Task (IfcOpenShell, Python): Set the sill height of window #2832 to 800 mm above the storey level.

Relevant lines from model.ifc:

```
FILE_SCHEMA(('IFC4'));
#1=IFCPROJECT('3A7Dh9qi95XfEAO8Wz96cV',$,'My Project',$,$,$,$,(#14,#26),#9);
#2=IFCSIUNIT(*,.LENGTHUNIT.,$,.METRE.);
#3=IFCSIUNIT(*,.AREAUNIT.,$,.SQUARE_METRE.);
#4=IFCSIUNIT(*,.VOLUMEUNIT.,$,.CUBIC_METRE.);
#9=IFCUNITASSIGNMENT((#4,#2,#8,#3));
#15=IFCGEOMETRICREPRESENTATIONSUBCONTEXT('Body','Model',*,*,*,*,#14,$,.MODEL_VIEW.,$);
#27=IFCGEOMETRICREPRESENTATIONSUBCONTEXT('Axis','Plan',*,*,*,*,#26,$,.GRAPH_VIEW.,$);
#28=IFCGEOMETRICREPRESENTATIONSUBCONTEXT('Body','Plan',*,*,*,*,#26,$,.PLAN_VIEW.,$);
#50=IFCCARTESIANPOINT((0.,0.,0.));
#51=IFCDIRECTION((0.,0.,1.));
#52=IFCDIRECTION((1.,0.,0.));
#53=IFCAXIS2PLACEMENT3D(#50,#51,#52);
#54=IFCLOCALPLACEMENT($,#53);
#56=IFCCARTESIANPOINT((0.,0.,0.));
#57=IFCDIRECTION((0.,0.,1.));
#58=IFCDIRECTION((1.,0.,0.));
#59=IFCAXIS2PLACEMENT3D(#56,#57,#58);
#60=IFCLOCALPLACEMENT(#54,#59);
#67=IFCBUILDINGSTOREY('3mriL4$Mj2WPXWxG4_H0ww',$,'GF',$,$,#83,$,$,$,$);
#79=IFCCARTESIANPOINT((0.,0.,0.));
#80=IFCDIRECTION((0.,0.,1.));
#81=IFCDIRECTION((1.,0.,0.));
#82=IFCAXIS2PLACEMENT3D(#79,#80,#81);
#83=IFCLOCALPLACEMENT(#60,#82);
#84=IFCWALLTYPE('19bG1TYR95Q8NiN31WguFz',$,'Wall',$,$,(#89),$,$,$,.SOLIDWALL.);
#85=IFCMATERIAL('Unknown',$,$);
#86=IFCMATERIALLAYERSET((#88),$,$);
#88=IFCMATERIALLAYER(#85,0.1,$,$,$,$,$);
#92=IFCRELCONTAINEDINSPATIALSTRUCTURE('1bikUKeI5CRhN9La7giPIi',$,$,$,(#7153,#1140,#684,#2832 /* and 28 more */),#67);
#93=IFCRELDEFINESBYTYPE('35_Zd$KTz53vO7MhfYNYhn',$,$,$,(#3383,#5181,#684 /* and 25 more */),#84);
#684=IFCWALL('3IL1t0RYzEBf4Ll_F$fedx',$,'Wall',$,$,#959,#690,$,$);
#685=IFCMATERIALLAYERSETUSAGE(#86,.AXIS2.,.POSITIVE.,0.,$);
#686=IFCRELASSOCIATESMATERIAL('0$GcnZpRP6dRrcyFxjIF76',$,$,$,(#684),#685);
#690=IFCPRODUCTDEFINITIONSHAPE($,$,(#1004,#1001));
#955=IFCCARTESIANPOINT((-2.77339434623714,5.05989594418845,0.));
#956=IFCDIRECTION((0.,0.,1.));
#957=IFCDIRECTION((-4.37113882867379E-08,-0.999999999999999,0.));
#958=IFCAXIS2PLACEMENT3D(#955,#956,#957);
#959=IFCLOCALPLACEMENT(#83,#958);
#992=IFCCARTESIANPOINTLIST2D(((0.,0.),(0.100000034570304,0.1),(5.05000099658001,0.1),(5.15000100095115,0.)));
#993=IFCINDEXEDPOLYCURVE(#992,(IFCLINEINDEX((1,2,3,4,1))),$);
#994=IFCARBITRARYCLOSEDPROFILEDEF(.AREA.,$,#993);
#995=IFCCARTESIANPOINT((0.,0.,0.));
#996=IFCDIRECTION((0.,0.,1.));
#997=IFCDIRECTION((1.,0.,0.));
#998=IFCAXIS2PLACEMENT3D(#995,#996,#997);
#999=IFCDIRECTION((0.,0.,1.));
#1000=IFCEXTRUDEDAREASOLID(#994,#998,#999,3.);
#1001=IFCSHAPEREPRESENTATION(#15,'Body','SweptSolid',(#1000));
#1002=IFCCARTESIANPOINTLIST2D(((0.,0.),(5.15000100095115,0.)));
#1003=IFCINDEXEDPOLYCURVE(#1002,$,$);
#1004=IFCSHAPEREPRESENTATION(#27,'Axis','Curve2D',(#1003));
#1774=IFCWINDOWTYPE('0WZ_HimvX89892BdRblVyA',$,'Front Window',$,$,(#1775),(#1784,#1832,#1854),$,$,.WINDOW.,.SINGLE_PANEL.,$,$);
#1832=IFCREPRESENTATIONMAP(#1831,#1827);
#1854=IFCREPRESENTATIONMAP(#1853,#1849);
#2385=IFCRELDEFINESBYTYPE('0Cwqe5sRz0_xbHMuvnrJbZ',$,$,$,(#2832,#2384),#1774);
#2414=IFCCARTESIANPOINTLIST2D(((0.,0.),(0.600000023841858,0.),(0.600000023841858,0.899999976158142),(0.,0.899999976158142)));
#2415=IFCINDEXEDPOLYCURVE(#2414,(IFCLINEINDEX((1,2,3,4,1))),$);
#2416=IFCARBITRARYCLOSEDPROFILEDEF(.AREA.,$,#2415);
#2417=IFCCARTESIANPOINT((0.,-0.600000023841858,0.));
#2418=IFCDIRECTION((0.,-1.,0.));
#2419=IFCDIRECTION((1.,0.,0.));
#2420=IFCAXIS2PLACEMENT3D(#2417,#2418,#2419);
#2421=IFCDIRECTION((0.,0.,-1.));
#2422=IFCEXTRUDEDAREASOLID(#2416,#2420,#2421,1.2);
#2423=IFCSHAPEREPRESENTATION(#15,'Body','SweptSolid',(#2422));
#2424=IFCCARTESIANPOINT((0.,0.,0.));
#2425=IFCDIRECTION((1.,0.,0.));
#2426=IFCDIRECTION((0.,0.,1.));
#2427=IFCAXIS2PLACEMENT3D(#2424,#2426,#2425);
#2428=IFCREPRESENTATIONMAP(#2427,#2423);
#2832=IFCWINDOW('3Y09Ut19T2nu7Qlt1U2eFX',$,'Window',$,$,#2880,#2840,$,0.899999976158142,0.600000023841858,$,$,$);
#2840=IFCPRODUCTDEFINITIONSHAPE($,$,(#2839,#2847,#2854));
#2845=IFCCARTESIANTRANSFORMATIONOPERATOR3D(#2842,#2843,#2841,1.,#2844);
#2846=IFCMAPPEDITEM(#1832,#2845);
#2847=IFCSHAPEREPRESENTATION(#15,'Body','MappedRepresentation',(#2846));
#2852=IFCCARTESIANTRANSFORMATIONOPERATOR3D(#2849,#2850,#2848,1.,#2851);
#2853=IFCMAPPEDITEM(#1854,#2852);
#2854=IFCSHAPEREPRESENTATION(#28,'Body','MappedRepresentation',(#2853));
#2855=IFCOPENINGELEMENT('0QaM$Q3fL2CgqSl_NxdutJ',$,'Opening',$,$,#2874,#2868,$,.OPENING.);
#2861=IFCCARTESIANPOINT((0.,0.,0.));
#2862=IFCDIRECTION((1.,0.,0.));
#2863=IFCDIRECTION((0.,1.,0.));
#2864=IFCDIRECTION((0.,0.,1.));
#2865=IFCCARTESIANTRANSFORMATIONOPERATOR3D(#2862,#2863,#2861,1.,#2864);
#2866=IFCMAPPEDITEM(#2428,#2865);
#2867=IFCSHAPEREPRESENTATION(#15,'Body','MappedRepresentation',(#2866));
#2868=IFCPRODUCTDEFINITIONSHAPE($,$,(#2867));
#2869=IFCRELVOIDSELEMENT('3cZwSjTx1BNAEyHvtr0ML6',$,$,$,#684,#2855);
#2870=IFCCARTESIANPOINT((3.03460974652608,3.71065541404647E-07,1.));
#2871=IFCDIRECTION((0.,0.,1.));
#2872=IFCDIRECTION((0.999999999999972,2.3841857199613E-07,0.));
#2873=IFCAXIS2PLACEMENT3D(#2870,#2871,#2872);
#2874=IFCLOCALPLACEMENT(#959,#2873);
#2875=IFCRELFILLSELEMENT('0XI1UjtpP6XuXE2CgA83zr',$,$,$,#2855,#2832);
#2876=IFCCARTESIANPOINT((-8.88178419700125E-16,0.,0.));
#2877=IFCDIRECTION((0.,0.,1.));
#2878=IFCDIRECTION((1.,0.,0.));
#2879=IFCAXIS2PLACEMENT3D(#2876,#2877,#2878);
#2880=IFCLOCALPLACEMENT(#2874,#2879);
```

```python
import numpy as np
import ifcopenshell
import ifcopenshell.api.geometry
import ifcopenshell.geom
import ifcopenshell.util.element
import ifcopenshell.util.placement
import ifcopenshell.util.shape
import ifcopenshell.util.unit

model = ifcopenshell.open("model.ifc")
unit_scale = ifcopenshell.util.unit.calculate_unit_scale(model)

window = model.by_id(2832)
opening = window.FillsVoids[0].RelatingOpeningElement
storey = ifcopenshell.util.element.get_container(window, ifc_class="IfcBuildingStorey")
level = ifcopenshell.util.placement.get_local_placement(storey.ObjectPlacement)[2, 3]

# The opening's origin need not be at the sill, so measure its lowest point.
shape = ifcopenshell.geom.create_shape(ifcopenshell.geom.settings(), opening)
bottom = ifcopenshell.util.shape.get_shape_bottom_elevation(shape, shape.geometry) / unit_scale
dz = level + 0.8 / unit_scale - bottom

shift = np.array([0.0, 0.0, dz])
# The window is placed relative to its opening, so it follows when the opening moves.
matrix = ifcopenshell.util.placement.get_local_placement(opening.ObjectPlacement)
matrix[:3, 3] += shift
ifcopenshell.api.geometry.edit_object_placement(
    model, product=opening, matrix=matrix, is_si=False, should_transform_children=True
)

print(f"moved by {dz * unit_scale:+.3f} m")

model.write("model_edited.ifc")
```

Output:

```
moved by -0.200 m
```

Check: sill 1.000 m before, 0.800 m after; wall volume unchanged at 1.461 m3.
